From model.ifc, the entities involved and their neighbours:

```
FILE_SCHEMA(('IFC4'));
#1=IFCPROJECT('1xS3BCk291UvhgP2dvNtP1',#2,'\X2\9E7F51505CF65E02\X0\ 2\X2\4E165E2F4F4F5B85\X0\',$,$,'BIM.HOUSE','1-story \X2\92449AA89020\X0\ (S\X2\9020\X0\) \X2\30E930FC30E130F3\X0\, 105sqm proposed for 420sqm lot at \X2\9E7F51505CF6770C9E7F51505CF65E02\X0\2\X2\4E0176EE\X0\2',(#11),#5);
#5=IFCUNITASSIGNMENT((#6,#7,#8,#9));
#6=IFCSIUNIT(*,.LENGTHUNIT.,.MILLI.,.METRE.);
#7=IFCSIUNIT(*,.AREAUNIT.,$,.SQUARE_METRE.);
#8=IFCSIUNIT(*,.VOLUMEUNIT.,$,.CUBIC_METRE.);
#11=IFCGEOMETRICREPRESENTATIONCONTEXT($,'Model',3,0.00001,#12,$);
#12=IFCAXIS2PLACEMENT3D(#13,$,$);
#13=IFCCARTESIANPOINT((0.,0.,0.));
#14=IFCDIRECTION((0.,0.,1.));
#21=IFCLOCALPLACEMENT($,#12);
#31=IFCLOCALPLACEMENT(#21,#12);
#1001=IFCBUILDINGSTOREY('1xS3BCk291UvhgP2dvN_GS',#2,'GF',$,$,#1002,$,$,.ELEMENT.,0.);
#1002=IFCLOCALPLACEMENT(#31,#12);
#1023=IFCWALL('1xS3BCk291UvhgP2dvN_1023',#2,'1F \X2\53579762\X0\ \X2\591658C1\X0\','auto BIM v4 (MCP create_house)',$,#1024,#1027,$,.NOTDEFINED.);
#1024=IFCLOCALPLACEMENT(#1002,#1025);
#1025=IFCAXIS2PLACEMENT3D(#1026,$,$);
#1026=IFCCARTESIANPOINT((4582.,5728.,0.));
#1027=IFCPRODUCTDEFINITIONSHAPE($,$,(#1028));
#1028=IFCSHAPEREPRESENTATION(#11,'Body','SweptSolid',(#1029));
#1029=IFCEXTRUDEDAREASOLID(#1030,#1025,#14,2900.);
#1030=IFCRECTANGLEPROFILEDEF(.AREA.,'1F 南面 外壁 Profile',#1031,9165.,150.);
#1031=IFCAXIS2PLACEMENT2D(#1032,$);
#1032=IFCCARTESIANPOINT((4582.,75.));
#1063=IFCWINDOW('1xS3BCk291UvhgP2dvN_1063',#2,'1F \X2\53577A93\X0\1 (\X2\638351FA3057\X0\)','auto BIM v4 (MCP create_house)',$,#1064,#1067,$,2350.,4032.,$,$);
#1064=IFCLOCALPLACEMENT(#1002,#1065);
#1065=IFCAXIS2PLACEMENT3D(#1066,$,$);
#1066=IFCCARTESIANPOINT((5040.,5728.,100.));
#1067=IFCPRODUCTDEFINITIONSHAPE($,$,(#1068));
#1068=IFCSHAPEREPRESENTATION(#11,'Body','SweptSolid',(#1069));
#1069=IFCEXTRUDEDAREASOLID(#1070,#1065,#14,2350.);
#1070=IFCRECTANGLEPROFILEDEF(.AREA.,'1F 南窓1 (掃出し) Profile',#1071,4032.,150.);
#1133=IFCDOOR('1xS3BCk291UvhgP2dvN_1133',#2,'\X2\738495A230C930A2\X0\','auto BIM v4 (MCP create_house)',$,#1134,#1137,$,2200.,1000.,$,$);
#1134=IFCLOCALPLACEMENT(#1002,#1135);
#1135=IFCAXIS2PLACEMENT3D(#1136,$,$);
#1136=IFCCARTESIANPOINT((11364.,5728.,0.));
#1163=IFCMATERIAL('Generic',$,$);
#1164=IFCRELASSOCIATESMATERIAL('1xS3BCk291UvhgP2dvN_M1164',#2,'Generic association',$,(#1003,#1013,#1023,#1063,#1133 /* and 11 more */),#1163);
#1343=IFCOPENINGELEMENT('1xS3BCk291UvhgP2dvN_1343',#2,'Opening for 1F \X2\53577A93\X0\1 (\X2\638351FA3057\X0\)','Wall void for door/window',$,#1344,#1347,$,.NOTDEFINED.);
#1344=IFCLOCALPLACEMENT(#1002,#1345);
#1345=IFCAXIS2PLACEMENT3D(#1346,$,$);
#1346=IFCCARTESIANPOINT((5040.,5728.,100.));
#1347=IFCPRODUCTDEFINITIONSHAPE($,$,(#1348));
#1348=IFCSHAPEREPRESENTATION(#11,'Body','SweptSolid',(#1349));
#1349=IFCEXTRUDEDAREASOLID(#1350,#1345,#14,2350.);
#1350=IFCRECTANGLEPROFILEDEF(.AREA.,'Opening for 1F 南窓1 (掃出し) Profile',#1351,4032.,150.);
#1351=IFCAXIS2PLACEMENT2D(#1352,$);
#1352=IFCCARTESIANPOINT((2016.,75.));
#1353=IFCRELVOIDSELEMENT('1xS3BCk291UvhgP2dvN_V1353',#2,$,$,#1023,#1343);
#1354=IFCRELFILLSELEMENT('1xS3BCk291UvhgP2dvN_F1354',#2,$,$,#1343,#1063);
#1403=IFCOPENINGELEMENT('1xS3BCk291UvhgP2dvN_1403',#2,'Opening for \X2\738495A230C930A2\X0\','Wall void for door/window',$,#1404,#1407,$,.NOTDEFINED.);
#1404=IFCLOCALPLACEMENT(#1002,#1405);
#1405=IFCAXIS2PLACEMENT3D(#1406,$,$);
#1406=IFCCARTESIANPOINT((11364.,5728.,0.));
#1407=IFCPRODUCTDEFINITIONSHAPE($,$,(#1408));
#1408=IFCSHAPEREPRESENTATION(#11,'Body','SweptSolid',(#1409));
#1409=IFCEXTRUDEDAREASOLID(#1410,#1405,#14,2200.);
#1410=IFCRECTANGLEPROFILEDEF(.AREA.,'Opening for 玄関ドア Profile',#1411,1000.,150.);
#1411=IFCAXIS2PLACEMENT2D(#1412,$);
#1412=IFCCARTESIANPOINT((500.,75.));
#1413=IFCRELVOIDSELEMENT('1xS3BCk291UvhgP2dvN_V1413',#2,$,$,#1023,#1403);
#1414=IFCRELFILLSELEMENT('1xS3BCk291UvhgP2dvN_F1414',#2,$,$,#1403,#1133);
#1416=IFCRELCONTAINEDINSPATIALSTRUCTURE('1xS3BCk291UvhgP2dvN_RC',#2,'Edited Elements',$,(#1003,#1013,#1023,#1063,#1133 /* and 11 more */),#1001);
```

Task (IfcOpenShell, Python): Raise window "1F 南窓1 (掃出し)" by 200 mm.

```python
import numpy as np
import ifcopenshell
import ifcopenshell.api.geometry
import ifcopenshell.util.placement
import ifcopenshell.util.unit

model = ifcopenshell.open("model.ifc")
unit_scale = ifcopenshell.util.unit.calculate_unit_scale(model)

window = model.by_guid("1xS3BCk291UvhgP2dvN_1063")
opening = window.FillsVoids[0].RelatingOpeningElement
dz = 0.2 / unit_scale

shift = np.array([0.0, 0.0, dz])
# The window is not placed relative to its opening, so move both.
for product in (opening, window):
    matrix = ifcopenshell.util.placement.get_local_placement(product.ObjectPlacement)
    matrix[:3, 3] += shift
    ifcopenshell.api.geometry.edit_object_placement(model, product=product, matrix=matrix, is_si=False)

print(f"moved by {dz * unit_scale:+.3f} m")

model.write("model_rev.ifc")
```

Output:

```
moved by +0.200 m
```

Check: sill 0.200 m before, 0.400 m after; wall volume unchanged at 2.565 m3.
